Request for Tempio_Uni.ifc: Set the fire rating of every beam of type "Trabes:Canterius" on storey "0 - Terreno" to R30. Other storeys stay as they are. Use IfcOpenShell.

First a look at what the model holds.

```python
import ifcopenshell
import ifcopenshell.util.element

model = ifcopenshell.open("Tempio_Uni.ifc")
print(model.schema)
storey = next(s for s in model.by_type("IfcBuildingStorey") if s.Name == "0 - Terreno")
beams = [e for e in ifcopenshell.util.element.get_decomposition(storey) if e.is_a("IfcBeam")]
seen = {}
for e in beams:
    element_type = ifcopenshell.util.element.get_type(e)
    key = (element_type.Name if element_type != e and element_type else None, ifcopenshell.util.element.get_pset(e, "Pset_BeamCommon", "FireRating"))
    seen[key] = seen.get(key, 0) + 1
for (name, value), count in sorted(seen.items(), key=str):
    print(count, "x", name, "|", value)
```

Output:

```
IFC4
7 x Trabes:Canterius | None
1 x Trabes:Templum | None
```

```python
import ifcopenshell
import ifcopenshell.api.pset
import ifcopenshell.util.element

model = ifcopenshell.open("Tempio_Uni.ifc")

storey = next(s for s in model.by_type("IfcBuildingStorey") if s.Name == "0 - Terreno")
beams = [e for e in ifcopenshell.util.element.get_decomposition(storey) if e.is_a("IfcBeam")]

count = 0
for e in beams:
    element_type = ifcopenshell.util.element.get_type(e)
    if element_type in (None, e) or element_type.Name != "Trabes:Canterius":
        continue
    # add_pset returns the element's existing set when there is one.
    pset = ifcopenshell.api.pset.add_pset(model, product=e, name="Pset_BeamCommon")
    ifcopenshell.api.pset.edit_pset(model, pset=pset, properties={"FireRating": "R30"})
    count += 1

print(count, "beams updated")

model.write("Tempio_Uni_updated.ifc")
```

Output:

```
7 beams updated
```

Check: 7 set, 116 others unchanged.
